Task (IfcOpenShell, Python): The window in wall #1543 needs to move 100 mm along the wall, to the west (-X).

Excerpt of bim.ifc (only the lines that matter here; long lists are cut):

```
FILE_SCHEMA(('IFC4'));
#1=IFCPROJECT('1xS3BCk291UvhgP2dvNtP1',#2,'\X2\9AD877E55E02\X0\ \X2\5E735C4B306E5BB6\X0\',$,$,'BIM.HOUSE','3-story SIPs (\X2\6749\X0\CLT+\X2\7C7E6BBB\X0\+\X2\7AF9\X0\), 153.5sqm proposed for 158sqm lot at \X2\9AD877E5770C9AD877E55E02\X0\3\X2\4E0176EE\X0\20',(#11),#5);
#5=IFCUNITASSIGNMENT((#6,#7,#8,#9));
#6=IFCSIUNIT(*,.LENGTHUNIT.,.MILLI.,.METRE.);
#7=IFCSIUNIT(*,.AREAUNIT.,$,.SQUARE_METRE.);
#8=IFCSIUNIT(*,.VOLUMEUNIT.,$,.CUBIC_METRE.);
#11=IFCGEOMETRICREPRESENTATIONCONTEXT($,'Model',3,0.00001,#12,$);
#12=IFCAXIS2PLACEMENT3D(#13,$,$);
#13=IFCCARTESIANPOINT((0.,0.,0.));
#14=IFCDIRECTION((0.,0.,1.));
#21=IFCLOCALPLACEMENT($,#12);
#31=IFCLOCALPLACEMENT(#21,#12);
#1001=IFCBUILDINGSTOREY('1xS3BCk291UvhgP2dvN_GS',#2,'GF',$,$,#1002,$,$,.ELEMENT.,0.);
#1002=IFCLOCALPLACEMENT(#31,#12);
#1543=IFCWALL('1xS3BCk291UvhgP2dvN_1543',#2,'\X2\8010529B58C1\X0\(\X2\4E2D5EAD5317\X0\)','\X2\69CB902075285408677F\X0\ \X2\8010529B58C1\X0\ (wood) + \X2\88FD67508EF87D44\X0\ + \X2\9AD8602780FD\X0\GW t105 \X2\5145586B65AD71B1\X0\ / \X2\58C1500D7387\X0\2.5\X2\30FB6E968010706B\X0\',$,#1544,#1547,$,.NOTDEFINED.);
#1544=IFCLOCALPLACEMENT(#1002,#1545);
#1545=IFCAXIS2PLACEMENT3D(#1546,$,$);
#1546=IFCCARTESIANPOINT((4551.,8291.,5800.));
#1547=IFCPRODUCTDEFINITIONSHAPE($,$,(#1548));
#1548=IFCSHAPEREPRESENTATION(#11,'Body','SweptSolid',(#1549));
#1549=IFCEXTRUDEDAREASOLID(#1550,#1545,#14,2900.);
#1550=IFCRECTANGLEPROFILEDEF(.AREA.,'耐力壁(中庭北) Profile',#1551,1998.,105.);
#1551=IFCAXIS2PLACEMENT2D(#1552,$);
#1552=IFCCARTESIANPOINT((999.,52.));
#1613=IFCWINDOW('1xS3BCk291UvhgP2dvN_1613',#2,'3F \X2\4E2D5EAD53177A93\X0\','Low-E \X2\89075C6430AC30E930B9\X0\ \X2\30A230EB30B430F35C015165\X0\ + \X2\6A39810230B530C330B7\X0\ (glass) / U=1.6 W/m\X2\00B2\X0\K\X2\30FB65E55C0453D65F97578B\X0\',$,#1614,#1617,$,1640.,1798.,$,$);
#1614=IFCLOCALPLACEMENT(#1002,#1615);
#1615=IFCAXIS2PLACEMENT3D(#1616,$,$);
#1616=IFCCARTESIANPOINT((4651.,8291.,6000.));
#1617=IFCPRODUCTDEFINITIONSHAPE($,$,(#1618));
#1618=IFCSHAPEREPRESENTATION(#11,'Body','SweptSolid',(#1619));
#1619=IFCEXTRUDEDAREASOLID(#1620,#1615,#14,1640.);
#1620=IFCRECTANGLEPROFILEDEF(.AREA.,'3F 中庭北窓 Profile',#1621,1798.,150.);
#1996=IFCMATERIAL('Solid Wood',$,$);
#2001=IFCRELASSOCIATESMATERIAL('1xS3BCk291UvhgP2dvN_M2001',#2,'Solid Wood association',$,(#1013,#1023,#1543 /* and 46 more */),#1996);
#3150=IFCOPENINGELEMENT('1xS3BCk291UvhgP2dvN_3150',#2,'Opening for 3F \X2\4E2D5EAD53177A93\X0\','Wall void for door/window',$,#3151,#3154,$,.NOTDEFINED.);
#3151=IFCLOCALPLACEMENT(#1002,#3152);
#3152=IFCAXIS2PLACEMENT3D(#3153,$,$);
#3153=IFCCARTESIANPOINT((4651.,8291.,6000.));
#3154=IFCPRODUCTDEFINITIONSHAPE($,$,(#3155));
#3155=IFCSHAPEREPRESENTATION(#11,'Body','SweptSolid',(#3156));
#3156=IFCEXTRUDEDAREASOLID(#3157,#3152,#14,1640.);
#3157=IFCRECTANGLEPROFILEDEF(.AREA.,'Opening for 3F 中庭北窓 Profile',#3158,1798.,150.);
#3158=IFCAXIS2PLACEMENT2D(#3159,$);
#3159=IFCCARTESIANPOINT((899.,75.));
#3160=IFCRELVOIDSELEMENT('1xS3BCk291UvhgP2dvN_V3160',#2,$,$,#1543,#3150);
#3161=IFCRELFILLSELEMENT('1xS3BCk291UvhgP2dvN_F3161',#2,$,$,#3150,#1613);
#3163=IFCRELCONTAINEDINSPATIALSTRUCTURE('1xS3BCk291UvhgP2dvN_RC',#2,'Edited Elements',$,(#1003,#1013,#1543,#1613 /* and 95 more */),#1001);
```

```python
import ifcopenshell
import ifcopenshell.api.geometry
import ifcopenshell.util.placement
import ifcopenshell.util.unit

model = ifcopenshell.open("bim.ifc")
unit_scale = ifcopenshell.util.unit.calculate_unit_scale(model)

window = model.by_guid("1xS3BCk291UvhgP2dvN_1613")
opening = window.FillsVoids[0].RelatingOpeningElement
wall = opening.VoidsElements[0].RelatingBuildingElement

wall_matrix = ifcopenshell.util.placement.get_local_placement(wall.ObjectPlacement)
shift = wall_matrix[:3, 0] * -0.1 / unit_scale
before = ifcopenshell.util.placement.get_local_placement(window.ObjectPlacement)[:3, 3].copy()

# The window is not placed relative to its opening, so move both.
for product in (opening, window):
    matrix = ifcopenshell.util.placement.get_local_placement(product.ObjectPlacement)
    matrix[:3, 3] += shift
    ifcopenshell.api.geometry.edit_object_placement(model, product=product, matrix=matrix, is_si=False)

after = ifcopenshell.util.placement.get_local_placement(window.ObjectPlacement)[:3, 3]
print("window moved by", (after - before).round(3) + 0.0)

model.write("bim-out.ifc")
```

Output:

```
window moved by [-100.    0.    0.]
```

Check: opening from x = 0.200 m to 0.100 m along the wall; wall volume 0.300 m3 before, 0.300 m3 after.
